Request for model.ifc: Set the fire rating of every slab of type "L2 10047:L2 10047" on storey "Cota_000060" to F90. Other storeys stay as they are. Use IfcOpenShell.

First a look at what the model holds.

```python
import ifcopenshell
import ifcopenshell.util.element

model = ifcopenshell.open("model.ifc")
print(model.schema)
storey = next(s for s in model.by_type("IfcBuildingStorey") if s.Name == "Cota_000060")
slabs = [e for e in ifcopenshell.util.element.get_decomposition(storey) if e.is_a("IfcSlab")]
seen = {}
for e in slabs:
    element_type = ifcopenshell.util.element.get_type(e)
    key = (element_type.Name if element_type != e and element_type else None, ifcopenshell.util.element.get_pset(e, "Pset_SlabCommon", "FireRating"))
    seen[key] = seen.get(key, 0) + 1
for (name, value), count in sorted(seen.items(), key=str):
    print(count, "x", name, "|", value)
```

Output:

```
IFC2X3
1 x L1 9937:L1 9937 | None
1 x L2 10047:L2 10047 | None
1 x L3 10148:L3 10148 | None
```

```python
import ifcopenshell
import ifcopenshell.api.pset
import ifcopenshell.util.element

model = ifcopenshell.open("model.ifc")

storey = next(s for s in model.by_type("IfcBuildingStorey") if s.Name == "Cota_000060")
slabs = [e for e in ifcopenshell.util.element.get_decomposition(storey) if e.is_a("IfcSlab")]

count = 0
for e in slabs:
    element_type = ifcopenshell.util.element.get_type(e)
    if element_type in (None, e) or element_type.Name != "L2 10047:L2 10047":
        continue
    # add_pset returns the element's existing set when there is one.
    pset = ifcopenshell.api.pset.add_pset(model, product=e, name="Pset_SlabCommon")
    ifcopenshell.api.pset.edit_pset(model, pset=pset, properties={"FireRating": "F90"})
    count += 1

print(count, "slabs updated")

model.write("model_edited.ifc")
```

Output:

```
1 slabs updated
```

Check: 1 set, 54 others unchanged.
